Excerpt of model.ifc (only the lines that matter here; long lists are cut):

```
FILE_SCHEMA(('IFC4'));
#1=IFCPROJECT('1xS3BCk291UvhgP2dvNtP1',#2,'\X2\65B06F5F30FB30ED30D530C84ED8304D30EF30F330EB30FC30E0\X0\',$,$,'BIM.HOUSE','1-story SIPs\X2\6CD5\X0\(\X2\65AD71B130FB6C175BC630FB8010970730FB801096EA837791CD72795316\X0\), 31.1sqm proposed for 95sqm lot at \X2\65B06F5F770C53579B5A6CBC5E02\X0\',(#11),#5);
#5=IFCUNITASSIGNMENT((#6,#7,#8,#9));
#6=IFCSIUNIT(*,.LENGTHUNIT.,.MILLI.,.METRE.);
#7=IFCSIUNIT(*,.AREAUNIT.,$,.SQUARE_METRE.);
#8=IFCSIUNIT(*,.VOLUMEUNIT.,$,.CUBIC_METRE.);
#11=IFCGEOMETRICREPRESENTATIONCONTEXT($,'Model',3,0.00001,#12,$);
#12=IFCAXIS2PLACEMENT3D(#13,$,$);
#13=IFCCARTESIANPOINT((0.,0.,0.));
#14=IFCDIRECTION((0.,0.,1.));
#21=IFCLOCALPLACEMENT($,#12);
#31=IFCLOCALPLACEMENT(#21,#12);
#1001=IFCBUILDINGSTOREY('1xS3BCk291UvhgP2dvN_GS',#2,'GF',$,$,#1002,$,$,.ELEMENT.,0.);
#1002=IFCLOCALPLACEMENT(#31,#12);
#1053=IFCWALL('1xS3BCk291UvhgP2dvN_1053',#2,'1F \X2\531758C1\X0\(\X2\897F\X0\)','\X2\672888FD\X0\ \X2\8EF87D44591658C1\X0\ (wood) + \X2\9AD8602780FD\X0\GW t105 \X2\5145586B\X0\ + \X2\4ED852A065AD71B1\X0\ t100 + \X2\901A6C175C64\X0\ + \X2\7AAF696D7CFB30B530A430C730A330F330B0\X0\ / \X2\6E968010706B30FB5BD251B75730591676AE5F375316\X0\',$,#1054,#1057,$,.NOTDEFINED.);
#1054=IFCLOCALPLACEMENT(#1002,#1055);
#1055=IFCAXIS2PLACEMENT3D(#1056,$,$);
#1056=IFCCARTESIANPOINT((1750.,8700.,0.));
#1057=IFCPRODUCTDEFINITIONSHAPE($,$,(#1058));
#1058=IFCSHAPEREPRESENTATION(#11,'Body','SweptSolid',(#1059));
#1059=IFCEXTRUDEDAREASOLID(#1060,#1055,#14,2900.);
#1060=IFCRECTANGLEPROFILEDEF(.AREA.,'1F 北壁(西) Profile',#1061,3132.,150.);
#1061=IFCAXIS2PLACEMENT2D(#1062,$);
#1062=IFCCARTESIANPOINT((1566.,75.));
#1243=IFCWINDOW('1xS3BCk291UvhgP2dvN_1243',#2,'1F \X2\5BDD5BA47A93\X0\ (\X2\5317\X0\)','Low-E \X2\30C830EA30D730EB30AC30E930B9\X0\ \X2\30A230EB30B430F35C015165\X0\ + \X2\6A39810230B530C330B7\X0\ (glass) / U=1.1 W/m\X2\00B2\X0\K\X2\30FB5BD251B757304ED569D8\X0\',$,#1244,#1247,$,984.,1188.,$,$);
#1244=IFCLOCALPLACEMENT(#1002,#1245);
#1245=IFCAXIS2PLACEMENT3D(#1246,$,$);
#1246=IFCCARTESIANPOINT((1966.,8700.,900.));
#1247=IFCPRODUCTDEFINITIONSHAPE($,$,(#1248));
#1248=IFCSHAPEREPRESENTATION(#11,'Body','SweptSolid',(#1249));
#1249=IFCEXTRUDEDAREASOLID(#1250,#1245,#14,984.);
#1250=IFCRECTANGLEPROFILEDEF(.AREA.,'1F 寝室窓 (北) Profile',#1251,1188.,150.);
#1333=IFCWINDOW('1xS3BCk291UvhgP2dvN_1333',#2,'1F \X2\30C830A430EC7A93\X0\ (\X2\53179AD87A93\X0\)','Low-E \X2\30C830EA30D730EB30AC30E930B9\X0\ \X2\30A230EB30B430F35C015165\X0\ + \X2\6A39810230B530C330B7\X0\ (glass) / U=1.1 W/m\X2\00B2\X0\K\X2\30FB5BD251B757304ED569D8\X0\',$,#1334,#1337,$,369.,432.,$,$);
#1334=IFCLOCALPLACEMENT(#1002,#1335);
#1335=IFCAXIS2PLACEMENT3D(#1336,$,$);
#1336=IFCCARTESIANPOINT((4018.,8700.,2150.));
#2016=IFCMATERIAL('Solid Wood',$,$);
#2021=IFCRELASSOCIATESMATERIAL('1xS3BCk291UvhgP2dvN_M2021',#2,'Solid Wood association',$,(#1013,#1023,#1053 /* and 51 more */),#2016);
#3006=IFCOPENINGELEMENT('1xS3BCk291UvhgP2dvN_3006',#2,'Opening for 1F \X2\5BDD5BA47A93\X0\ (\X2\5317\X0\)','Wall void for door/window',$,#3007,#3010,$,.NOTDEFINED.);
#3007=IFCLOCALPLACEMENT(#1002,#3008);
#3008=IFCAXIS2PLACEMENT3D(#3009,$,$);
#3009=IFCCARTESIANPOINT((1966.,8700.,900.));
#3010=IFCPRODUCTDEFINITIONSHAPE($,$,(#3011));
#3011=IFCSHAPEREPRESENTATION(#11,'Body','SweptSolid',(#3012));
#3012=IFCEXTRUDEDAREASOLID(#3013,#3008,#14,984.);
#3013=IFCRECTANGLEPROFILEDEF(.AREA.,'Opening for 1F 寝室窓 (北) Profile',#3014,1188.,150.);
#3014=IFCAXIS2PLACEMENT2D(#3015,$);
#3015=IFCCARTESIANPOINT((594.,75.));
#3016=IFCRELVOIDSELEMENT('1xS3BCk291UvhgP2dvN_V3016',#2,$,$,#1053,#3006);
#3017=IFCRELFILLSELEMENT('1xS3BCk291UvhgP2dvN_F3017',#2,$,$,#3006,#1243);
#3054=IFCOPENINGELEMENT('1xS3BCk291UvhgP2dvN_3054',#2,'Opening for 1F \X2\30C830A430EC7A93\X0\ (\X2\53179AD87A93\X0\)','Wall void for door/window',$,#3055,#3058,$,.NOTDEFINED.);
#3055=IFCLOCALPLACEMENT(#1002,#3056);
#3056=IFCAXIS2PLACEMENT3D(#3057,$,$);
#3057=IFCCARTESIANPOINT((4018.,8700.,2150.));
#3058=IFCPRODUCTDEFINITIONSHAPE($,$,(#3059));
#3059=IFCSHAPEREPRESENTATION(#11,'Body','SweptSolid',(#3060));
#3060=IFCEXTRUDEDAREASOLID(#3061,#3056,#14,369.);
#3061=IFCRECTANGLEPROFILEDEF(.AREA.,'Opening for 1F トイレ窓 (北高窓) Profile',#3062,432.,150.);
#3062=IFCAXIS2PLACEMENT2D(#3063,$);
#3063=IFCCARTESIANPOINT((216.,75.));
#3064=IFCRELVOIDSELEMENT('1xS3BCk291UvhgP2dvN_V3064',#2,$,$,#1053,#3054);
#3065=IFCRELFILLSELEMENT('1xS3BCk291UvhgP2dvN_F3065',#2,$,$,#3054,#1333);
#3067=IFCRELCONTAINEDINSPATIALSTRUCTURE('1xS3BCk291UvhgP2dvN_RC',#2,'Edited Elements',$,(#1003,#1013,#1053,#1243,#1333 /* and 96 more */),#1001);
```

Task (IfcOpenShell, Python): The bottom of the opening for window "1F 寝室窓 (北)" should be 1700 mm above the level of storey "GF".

```python
import numpy as np
import ifcopenshell
import ifcopenshell.api.geometry
import ifcopenshell.geom
import ifcopenshell.util.element
import ifcopenshell.util.placement
import ifcopenshell.util.shape
import ifcopenshell.util.unit

model = ifcopenshell.open("model.ifc")
unit_scale = ifcopenshell.util.unit.calculate_unit_scale(model)

window = model.by_id(1243)
opening = window.FillsVoids[0].RelatingOpeningElement
storey = ifcopenshell.util.element.get_container(window, ifc_class="IfcBuildingStorey")
level = ifcopenshell.util.placement.get_local_placement(storey.ObjectPlacement)[2, 3]

# The opening's origin need not be at the sill, so measure its lowest point.
shape = ifcopenshell.geom.create_shape(ifcopenshell.geom.settings(), opening)
bottom = ifcopenshell.util.shape.get_shape_bottom_elevation(shape, shape.geometry) / unit_scale
dz = level + 1.7 / unit_scale - bottom

shift = np.array([0.0, 0.0, dz])
# The window is not placed relative to its opening, so move both.
for product in (opening, window):
    matrix = ifcopenshell.util.placement.get_local_placement(product.ObjectPlacement)
    matrix[:3, 3] += shift
    ifcopenshell.api.geometry.edit_object_placement(model, product=product, matrix=matrix, is_si=False)

print(f"moved by {dz * unit_scale:+.3f} m")

model.write("model_updated.ifc")
```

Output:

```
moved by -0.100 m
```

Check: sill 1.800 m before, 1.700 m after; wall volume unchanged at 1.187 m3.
